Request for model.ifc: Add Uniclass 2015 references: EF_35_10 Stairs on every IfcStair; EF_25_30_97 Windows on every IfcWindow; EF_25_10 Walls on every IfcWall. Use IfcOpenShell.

First a look at what the model holds.

```python
import ifcopenshell

model = ifcopenshell.open("model.ifc")
print(model.schema)
print("classifications:", [c.Name for c in model.by_type("IfcClassification")])
for ifc_class in ("IfcDoor", "IfcRoof", "IfcStair", "IfcWall", "IfcWindow"):
    print(ifc_class, len(model.by_type(ifc_class)))
```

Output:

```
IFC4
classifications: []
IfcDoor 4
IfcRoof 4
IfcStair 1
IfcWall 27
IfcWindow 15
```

```python
import ifcopenshell
import ifcopenshell.api.classification

model = ifcopenshell.open("model.ifc")

system = ifcopenshell.api.classification.add_classification(model, classification="Uniclass 2015")

codes = {
    "IfcStair": ("EF_35_10", "Stairs"),
    "IfcWindow": ("EF_25_30_97", "Windows"),
    "IfcWall": ("EF_25_10", "Walls"),
}
for ifc_class, (code, name) in codes.items():
    products = model.by_type(ifc_class)
    ifcopenshell.api.classification.add_reference(
        model, products=products, classification=system, identification=code, name=name
    )
    print(code, len(products))

model.write("model_rev.ifc")
```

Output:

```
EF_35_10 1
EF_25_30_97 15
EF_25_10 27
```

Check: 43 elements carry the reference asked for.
